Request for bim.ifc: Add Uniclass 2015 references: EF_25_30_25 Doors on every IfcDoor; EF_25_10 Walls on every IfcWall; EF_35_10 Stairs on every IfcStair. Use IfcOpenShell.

First a look at what the model holds.

```python
import ifcopenshell

model = ifcopenshell.open("bim.ifc")
print(model.schema)
print("classifications:", [c.Name for c in model.by_type("IfcClassification")])
for ifc_class in ("IfcDoor", "IfcRoof", "IfcStair", "IfcWall", "IfcWindow"):
    print(ifc_class, len(model.by_type(ifc_class)))
```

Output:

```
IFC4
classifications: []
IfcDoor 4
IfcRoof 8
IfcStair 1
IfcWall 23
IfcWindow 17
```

```python
import ifcopenshell
import ifcopenshell.api.classification

model = ifcopenshell.open("bim.ifc")

system = ifcopenshell.api.classification.add_classification(model, classification="Uniclass 2015")

codes = {
    "IfcDoor": ("EF_25_30_25", "Doors"),
    "IfcWall": ("EF_25_10", "Walls"),
    "IfcStair": ("EF_35_10", "Stairs"),
}
for ifc_class, (code, name) in codes.items():
    products = model.by_type(ifc_class)
    ifcopenshell.api.classification.add_reference(
        model, products=products, classification=system, identification=code, name=name
    )
    print(code, len(products))

model.write("bim_updated.ifc")
```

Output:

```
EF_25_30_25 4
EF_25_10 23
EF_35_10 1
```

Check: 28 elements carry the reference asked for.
